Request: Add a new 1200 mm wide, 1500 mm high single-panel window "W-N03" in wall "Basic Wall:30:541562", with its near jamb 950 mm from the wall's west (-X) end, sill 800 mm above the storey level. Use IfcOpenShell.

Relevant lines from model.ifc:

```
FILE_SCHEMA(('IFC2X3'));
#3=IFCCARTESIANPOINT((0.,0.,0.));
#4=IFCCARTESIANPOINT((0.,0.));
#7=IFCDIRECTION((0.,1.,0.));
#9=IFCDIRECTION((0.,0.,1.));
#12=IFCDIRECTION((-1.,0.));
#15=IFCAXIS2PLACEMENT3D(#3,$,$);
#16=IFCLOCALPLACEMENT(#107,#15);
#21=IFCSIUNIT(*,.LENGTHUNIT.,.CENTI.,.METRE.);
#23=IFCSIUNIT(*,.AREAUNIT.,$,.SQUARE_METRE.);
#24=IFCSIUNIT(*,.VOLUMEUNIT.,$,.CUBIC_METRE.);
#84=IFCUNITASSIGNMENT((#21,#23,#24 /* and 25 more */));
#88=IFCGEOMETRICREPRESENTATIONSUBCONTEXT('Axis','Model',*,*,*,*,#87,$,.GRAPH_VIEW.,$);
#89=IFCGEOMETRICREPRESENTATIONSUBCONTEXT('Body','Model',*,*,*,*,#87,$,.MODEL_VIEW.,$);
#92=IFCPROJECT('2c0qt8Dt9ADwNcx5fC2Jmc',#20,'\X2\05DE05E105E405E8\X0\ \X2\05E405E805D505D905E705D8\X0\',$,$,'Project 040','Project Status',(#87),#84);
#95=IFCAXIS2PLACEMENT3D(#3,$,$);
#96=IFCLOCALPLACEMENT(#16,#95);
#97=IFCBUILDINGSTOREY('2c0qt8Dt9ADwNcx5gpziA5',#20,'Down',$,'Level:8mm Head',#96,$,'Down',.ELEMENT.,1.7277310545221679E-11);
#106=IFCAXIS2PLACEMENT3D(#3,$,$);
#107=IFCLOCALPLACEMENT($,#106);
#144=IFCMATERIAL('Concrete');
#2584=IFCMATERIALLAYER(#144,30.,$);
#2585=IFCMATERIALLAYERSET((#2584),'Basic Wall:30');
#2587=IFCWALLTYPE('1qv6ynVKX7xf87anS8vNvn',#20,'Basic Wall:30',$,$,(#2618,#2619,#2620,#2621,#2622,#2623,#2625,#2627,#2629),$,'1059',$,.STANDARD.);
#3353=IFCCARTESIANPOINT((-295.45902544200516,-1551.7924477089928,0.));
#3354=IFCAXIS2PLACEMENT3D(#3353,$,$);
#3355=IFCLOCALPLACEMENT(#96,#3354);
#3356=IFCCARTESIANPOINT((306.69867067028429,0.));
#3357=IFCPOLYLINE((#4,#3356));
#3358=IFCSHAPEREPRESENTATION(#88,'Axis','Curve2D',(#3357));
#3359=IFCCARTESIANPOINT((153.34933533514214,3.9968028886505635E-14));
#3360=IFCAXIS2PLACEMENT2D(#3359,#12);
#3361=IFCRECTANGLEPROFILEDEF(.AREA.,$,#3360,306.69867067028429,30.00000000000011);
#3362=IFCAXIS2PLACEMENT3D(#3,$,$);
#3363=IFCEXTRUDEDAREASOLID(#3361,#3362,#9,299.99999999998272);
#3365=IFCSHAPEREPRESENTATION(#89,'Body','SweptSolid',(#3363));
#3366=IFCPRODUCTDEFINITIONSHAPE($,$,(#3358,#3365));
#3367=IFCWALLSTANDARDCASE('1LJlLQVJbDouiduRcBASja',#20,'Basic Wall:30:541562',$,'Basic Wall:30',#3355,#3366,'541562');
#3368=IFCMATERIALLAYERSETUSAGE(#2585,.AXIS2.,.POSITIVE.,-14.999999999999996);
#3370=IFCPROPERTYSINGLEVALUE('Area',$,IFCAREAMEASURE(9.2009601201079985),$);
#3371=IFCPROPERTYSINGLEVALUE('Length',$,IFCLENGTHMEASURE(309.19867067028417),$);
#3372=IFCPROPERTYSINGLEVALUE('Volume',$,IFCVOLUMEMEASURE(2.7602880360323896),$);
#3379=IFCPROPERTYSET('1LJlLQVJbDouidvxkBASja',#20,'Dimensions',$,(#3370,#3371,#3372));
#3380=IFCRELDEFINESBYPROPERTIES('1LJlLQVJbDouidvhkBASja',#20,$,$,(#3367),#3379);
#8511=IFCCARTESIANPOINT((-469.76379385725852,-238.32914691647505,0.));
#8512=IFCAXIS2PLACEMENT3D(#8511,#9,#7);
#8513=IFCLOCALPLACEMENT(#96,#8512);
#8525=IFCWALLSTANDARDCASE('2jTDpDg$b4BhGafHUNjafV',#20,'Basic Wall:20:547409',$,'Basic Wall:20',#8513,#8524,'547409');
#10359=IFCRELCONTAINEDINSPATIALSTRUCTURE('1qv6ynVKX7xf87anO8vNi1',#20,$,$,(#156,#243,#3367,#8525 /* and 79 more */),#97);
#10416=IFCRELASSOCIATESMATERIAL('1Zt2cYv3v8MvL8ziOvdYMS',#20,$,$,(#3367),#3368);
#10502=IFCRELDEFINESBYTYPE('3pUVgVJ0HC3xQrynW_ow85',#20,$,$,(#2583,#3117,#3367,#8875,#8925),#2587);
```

```python
import numpy as np
import ifcopenshell
import ifcopenshell.api.feature
import ifcopenshell.api.geometry
import ifcopenshell.api.pset
import ifcopenshell.api.root
import ifcopenshell.api.spatial
import ifcopenshell.api.type
import ifcopenshell.geom
import ifcopenshell.util.element
import ifcopenshell.util.placement
import ifcopenshell.util.representation
import ifcopenshell.util.shape
import ifcopenshell.util.unit

model = ifcopenshell.open("model.ifc")
unit_scale = ifcopenshell.util.unit.calculate_unit_scale(model)
area_scale = ifcopenshell.util.unit.calculate_unit_scale(model, "AREAUNIT")
volume_scale = ifcopenshell.util.unit.calculate_unit_scale(model, "VOLUMEUNIT")
settings = ifcopenshell.geom.settings()


def volume(element):
    """Net volume in cubic metres, openings subtracted."""
    shape = ifcopenshell.geom.create_shape(settings, element)
    return ifcopenshell.util.shape.get_volume(shape.geometry)


wall = model.by_id(3367)
storey = ifcopenshell.util.element.get_container(wall, ifc_class="IfcBuildingStorey")
context = ifcopenshell.util.representation.get_context(model, "Model", "Body", "MODEL_VIEW")
before = volume(wall)

width, height, from_end, sill = 1.2, 1.5, 0.95, 0.8  # metres

# The wall runs along its own X axis, and the end named is its -X end.
wall_shape = ifcopenshell.geom.create_shape(settings, wall)
x, y, z = ifcopenshell.util.shape.get_vertices(wall_shape.geometry).T
start = x.min() + from_end
face, thickness = float(y.min()), float(y.max() - y.min())
wall_matrix = ifcopenshell.util.placement.get_local_placement(wall.ObjectPlacement)
level = ifcopenshell.util.placement.get_local_placement(storey.ObjectPlacement)[2, 3]


def in_wall(x, y):
    """Placement at x, y metres in the wall's axes, at sill height."""
    matrix = wall_matrix.copy()
    matrix[:, 3] = wall_matrix @ np.array([x / unit_scale, y / unit_scale, 0.0, 1.0])
    matrix[2, 3] = level + sill / unit_scale
    return matrix


# Opening: a box that overshoots both wall faces by 50 mm.
opening = ifcopenshell.api.root.create_entity(model, ifc_class="IfcOpeningElement")
box = ifcopenshell.api.geometry.add_wall_representation(
    model, context=context, length=width, height=height, thickness=thickness + 0.1
)
ifcopenshell.api.geometry.assign_representation(model, product=opening, representation=box)
ifcopenshell.api.geometry.edit_object_placement(model, product=opening, matrix=in_wall(start, face - 0.05), is_si=False)
ifcopenshell.api.feature.add_feature(model, feature=opening, element=wall)

window = ifcopenshell.api.root.create_entity(model, ifc_class="IfcWindow", name="W-N03")
window.OverallWidth, window.OverallHeight = width / unit_scale, height / unit_scale
body = ifcopenshell.api.geometry.add_window_representation(
    model,
    context=context,
    overall_width=window.OverallWidth,
    overall_height=window.OverallHeight,
    partition_type="SINGLE_PANEL",
)
ifcopenshell.api.geometry.assign_representation(model, product=window, representation=body)
ifcopenshell.api.spatial.assign_container(model, products=[window], relating_structure=storey)
fills = ifcopenshell.api.feature.add_filling(model, opening=opening, element=window)
fills.OwnerHistory = window.OwnerHistory  # required in IFC2X3

# IFC2X3 keeps the operation on the window style.
style = ifcopenshell.api.root.create_entity(model, ifc_class="IfcWindowStyle", name="W-N03")
style.OperationType, style.ConstructionType = "SINGLE_PANEL", "NOTDEFINED"
style.ParameterTakesPrecedence = style.Sizeable = False
ifcopenshell.api.type.assign_type(model, related_objects=[window], relating_type=style)

# Centre the window in the wall's thickness.
ifcopenshell.api.geometry.edit_object_placement(model, product=window, matrix=in_wall(start, face), is_si=False)
window_shape = ifcopenshell.geom.create_shape(settings, window)
depth = ifcopenshell.util.shape.get_vertices(window_shape.geometry)[:, 1]
offset = face + thickness / 2 - (depth.min() + depth.max()) / 2
ifcopenshell.api.geometry.edit_object_placement(model, product=window, matrix=in_wall(start, offset), is_si=False)

after = volume(wall)

# Update the wall's stored quantities.
pset = model.by_id(ifcopenshell.util.element.get_pset(wall, "Dimensions", should_inherit=False)["id"])
ifcopenshell.api.pset.edit_pset(model, pset=pset, properties={
    "Area": model.create_entity("IfcAreaMeasure", after / thickness / area_scale),
    "Volume": model.create_entity("IfcVolumeMeasure", after / volume_scale),
})

print(f"wall volume {before:.3f} -> {after:.3f} m3")

model.write("model-out.ifc")
```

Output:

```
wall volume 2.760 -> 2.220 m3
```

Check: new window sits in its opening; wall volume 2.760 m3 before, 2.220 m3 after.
